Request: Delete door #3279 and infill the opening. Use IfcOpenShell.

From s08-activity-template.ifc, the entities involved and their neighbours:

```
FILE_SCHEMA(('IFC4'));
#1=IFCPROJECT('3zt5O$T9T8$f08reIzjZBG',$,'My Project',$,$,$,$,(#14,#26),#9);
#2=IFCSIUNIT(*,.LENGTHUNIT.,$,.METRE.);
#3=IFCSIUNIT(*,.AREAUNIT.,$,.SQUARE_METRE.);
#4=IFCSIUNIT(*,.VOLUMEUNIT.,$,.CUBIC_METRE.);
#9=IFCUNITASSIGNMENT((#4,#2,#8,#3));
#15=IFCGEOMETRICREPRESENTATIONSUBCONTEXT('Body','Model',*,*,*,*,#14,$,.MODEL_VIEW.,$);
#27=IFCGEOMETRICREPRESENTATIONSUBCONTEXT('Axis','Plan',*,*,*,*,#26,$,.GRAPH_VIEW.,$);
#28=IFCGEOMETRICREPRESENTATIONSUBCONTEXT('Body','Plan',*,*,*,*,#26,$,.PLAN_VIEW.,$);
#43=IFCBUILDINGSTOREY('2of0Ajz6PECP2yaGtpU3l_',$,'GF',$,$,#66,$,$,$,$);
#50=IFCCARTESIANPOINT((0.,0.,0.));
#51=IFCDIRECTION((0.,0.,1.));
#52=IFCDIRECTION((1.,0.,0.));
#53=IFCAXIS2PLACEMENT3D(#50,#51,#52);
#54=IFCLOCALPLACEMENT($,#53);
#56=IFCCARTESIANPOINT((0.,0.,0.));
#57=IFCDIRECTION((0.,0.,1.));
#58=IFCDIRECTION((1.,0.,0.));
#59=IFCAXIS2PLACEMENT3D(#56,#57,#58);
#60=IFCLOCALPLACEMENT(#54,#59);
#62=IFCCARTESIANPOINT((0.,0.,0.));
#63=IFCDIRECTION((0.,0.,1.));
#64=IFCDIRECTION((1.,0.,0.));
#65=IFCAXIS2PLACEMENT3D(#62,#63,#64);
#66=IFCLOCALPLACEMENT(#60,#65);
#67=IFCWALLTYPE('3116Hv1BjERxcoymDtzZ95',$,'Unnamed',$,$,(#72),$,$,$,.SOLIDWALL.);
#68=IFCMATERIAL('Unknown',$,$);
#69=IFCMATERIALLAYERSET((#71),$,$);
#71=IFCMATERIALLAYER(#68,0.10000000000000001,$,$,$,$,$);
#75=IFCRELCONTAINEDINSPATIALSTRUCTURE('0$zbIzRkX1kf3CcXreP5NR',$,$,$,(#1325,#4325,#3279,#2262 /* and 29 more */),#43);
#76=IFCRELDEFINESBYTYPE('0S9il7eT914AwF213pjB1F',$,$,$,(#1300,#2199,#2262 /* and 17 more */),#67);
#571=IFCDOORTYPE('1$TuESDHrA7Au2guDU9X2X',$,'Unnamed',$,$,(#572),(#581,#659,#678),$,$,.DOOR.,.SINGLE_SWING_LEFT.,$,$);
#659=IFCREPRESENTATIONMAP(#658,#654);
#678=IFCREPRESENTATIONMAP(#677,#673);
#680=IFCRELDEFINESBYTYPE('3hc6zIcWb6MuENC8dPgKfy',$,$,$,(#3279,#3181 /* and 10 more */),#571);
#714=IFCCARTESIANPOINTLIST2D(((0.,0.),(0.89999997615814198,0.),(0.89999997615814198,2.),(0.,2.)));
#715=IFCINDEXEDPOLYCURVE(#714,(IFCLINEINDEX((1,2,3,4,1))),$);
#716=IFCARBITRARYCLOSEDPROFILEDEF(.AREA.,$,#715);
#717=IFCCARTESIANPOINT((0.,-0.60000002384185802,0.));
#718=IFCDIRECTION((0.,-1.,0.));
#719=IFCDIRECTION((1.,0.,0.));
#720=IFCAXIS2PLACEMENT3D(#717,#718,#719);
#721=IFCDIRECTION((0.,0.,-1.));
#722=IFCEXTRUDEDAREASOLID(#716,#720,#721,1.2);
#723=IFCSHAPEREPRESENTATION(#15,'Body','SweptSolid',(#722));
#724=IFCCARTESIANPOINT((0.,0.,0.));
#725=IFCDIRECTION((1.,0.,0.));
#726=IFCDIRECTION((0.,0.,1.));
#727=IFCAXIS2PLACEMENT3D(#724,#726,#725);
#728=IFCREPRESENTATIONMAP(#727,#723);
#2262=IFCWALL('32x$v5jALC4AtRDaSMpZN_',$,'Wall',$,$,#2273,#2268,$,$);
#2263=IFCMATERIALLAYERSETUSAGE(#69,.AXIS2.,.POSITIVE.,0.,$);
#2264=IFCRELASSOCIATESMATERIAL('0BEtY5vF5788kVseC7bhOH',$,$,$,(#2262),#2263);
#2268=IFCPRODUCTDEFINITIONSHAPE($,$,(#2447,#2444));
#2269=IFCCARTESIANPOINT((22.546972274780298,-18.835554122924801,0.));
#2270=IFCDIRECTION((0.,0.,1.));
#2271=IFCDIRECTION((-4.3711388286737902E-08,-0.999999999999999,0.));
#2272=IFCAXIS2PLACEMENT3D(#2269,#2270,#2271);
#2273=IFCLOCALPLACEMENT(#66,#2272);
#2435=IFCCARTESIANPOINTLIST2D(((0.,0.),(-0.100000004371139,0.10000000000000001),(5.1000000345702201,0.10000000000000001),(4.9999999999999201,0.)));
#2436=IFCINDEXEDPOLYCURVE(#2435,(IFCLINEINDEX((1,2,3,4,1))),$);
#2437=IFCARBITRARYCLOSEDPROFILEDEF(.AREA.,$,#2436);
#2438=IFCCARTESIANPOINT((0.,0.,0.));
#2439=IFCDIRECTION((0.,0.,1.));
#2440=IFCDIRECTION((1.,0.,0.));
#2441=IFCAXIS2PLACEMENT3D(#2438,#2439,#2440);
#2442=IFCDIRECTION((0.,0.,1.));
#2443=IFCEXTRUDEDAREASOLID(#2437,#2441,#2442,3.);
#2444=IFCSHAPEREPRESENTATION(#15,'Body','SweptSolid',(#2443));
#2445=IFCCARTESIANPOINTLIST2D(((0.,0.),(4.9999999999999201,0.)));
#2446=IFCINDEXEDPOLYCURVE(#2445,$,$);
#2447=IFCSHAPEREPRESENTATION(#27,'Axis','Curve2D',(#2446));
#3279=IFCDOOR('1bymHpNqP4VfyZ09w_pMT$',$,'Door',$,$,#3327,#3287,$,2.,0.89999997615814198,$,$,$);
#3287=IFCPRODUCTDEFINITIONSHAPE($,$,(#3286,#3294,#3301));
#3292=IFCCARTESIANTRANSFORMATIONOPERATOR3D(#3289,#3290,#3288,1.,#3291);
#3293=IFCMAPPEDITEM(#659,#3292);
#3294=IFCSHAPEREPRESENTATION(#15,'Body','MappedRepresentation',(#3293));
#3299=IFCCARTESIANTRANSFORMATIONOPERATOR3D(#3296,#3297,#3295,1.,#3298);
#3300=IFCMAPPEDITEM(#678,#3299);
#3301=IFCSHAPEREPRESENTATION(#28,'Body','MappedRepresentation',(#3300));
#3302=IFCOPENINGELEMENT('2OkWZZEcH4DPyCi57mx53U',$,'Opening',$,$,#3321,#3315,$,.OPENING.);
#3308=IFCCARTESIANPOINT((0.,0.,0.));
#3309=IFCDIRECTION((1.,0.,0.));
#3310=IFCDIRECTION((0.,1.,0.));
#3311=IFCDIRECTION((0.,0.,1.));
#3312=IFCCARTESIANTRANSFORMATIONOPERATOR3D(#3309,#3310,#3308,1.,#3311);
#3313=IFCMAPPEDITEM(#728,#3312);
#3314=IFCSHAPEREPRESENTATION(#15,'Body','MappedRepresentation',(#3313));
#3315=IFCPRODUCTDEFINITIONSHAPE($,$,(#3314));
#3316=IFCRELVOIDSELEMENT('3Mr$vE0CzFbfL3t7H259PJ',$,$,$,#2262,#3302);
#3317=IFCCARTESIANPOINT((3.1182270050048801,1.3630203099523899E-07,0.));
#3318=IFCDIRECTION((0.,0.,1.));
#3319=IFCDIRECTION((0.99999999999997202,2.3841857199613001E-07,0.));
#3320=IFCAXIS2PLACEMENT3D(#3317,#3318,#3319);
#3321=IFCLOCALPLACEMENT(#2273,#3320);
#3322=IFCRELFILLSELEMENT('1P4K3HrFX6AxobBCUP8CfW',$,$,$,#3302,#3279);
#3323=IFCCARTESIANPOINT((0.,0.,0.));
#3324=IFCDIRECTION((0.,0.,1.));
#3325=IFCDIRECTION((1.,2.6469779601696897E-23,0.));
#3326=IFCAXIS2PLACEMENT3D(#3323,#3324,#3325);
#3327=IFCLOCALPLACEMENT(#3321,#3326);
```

```python
import ifcopenshell
import ifcopenshell.api.feature
import ifcopenshell.api.root
import ifcopenshell.geom
import ifcopenshell.util.shape

model = ifcopenshell.open("s08-activity-template.ifc")
settings = ifcopenshell.geom.settings()


def volume(element):
    """Net volume in cubic metres, openings subtracted."""
    shape = ifcopenshell.geom.create_shape(settings, element)
    return ifcopenshell.util.shape.get_volume(shape.geometry)


door = model.by_id(3279)
opening = door.FillsVoids[0].RelatingOpeningElement
wall = opening.VoidsElements[0].RelatingBuildingElement
before = volume(wall)

ifcopenshell.api.root.remove_product(model, product=door)
ifcopenshell.api.feature.remove_feature(model, feature=opening)

after = volume(wall)

print(f"wall volume {before:.3f} -> {after:.3f} m3")

model.write("s08-activity-template_edited.ifc")
```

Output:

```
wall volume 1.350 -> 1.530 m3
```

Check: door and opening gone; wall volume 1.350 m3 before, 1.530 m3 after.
